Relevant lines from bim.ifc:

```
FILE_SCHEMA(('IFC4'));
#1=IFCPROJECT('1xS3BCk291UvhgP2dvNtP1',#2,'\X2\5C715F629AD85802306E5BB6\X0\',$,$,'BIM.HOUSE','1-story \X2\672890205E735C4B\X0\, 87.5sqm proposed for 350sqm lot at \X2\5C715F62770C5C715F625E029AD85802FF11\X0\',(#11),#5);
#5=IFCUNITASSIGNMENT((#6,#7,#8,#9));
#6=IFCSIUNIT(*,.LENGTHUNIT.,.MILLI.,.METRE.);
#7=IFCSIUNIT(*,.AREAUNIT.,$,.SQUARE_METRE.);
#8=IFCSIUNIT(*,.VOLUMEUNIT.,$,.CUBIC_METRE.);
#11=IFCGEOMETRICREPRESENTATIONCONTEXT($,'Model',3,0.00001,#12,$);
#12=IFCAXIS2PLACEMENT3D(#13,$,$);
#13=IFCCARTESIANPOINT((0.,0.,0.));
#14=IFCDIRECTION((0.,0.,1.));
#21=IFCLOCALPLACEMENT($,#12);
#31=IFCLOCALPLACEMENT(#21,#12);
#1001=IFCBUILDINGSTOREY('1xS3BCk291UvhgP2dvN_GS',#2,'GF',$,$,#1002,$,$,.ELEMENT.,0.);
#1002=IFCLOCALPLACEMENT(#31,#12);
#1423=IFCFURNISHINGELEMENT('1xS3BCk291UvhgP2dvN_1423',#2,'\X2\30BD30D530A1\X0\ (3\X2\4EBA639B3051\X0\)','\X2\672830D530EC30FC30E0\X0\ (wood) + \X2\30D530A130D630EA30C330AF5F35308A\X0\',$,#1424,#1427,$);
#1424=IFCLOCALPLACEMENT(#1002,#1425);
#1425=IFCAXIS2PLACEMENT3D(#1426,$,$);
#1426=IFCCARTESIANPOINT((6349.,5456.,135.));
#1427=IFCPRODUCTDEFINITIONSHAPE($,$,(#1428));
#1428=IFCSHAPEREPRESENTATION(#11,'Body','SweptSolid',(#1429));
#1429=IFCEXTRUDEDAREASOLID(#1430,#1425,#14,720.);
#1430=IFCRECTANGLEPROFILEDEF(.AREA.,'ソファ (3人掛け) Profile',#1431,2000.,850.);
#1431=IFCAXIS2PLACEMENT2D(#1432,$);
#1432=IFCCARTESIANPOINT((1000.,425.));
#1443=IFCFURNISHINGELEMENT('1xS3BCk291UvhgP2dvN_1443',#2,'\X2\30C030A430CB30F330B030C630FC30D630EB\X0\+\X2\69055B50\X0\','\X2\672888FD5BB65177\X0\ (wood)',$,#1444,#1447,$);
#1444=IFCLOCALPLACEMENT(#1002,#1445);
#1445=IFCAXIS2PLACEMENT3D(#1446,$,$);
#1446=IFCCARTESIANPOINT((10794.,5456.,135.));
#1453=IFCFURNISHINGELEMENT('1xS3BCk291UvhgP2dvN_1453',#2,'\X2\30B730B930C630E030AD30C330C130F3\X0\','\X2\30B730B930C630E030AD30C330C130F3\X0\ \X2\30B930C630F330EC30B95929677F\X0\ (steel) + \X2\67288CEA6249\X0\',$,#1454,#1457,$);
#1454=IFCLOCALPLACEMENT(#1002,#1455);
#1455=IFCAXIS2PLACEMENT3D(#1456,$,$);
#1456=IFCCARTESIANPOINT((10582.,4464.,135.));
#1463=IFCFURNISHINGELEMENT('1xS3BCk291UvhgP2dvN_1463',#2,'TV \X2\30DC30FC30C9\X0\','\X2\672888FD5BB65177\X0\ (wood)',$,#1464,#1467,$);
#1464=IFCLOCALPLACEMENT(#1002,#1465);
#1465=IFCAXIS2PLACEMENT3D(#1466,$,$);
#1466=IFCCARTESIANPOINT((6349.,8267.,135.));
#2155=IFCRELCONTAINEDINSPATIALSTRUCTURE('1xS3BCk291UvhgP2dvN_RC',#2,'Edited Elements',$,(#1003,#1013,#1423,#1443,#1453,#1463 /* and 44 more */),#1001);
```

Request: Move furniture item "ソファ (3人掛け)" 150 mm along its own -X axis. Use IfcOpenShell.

```python
import ifcopenshell
import ifcopenshell.api.geometry
import ifcopenshell.util.placement

model = ifcopenshell.open("bim.ifc")

item = model.by_guid("1xS3BCk291UvhgP2dvN_1423")
matrix = ifcopenshell.util.placement.get_local_placement(item.ObjectPlacement)
matrix[:3, 3] -= matrix[:3, 0] * 150.0
ifcopenshell.api.geometry.edit_object_placement(model, product=item, matrix=matrix, is_si=False)

print(ifcopenshell.util.placement.get_local_placement(item.ObjectPlacement).round(3) + 0.0)

model.write("bim_rev.ifc")
```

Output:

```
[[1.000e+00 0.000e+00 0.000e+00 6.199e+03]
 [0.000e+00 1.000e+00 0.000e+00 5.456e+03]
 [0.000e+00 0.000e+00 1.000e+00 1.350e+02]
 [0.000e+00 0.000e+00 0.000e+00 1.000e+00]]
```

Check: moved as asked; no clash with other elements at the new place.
